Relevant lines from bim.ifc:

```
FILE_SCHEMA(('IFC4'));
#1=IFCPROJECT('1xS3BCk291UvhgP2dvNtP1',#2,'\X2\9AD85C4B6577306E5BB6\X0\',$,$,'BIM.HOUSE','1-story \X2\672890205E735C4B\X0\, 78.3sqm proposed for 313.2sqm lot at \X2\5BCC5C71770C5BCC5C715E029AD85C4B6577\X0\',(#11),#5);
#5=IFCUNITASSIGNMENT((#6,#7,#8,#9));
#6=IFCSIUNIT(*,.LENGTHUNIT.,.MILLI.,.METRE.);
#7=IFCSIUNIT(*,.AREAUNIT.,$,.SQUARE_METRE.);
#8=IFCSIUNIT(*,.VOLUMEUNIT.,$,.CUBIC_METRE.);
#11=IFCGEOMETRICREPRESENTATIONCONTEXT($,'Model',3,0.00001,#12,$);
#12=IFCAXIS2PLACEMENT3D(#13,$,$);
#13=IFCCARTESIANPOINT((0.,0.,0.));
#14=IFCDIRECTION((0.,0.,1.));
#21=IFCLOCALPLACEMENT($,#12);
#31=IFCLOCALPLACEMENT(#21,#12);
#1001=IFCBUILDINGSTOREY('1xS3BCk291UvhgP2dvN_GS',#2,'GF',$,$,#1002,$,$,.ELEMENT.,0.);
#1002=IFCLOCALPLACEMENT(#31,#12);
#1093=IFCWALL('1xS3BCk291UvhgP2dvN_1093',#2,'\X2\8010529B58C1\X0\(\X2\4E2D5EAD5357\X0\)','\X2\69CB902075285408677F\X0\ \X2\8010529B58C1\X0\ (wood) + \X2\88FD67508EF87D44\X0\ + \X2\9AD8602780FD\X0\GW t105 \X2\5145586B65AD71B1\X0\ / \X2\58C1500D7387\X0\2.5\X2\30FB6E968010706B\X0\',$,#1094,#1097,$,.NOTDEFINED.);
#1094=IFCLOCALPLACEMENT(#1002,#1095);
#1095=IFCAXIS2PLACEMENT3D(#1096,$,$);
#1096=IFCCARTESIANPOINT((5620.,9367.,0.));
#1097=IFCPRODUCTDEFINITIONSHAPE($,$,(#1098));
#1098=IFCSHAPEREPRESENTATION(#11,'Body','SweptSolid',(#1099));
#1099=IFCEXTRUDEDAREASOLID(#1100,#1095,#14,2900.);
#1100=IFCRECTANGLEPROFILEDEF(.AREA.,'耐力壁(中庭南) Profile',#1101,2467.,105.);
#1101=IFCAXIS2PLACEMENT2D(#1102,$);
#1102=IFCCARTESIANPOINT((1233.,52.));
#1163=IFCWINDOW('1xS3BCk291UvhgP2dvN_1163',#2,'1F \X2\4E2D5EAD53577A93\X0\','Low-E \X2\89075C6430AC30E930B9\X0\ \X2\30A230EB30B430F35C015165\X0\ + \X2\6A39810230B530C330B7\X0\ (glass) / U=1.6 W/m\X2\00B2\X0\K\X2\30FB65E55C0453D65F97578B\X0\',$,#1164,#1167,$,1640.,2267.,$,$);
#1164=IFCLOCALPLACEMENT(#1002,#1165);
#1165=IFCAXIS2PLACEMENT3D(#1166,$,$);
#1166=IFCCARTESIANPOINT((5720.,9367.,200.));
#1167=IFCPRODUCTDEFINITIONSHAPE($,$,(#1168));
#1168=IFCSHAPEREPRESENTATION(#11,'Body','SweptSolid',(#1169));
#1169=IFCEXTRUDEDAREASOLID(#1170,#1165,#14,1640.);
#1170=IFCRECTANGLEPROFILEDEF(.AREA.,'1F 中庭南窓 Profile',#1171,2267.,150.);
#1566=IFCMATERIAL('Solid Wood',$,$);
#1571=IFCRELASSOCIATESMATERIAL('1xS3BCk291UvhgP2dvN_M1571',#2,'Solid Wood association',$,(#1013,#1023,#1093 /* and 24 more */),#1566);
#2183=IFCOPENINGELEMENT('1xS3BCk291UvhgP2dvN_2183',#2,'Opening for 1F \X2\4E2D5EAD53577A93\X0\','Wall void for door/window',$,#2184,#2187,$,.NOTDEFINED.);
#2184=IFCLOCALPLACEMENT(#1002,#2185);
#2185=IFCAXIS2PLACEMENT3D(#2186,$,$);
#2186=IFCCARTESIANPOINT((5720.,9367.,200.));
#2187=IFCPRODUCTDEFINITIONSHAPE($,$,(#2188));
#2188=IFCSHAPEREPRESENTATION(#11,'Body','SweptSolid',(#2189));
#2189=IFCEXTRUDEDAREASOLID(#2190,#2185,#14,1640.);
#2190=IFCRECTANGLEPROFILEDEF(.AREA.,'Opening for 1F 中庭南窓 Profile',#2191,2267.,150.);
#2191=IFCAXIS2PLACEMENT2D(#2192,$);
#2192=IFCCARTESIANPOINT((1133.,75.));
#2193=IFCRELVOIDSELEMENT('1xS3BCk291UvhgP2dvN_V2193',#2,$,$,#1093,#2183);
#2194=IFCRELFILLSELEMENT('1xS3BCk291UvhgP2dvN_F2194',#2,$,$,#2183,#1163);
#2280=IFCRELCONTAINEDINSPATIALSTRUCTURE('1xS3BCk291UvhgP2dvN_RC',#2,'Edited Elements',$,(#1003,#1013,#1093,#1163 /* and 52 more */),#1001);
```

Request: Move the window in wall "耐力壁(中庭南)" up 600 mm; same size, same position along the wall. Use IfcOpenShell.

```python
import numpy as np
import ifcopenshell
import ifcopenshell.api.geometry
import ifcopenshell.util.placement
import ifcopenshell.util.unit

model = ifcopenshell.open("bim.ifc")
unit_scale = ifcopenshell.util.unit.calculate_unit_scale(model)

window = model.by_guid("1xS3BCk291UvhgP2dvN_1163")
opening = window.FillsVoids[0].RelatingOpeningElement
dz = 0.6 / unit_scale

shift = np.array([0.0, 0.0, dz])
# The window is not placed relative to its opening, so move both.
for product in (opening, window):
    matrix = ifcopenshell.util.placement.get_local_placement(product.ObjectPlacement)
    matrix[:3, 3] += shift
    ifcopenshell.api.geometry.edit_object_placement(model, product=product, matrix=matrix, is_si=False)

print(f"moved by {dz * unit_scale:+.3f} m")

model.write("bim_edited.ifc")
```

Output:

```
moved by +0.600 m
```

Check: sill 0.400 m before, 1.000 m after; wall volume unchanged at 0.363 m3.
